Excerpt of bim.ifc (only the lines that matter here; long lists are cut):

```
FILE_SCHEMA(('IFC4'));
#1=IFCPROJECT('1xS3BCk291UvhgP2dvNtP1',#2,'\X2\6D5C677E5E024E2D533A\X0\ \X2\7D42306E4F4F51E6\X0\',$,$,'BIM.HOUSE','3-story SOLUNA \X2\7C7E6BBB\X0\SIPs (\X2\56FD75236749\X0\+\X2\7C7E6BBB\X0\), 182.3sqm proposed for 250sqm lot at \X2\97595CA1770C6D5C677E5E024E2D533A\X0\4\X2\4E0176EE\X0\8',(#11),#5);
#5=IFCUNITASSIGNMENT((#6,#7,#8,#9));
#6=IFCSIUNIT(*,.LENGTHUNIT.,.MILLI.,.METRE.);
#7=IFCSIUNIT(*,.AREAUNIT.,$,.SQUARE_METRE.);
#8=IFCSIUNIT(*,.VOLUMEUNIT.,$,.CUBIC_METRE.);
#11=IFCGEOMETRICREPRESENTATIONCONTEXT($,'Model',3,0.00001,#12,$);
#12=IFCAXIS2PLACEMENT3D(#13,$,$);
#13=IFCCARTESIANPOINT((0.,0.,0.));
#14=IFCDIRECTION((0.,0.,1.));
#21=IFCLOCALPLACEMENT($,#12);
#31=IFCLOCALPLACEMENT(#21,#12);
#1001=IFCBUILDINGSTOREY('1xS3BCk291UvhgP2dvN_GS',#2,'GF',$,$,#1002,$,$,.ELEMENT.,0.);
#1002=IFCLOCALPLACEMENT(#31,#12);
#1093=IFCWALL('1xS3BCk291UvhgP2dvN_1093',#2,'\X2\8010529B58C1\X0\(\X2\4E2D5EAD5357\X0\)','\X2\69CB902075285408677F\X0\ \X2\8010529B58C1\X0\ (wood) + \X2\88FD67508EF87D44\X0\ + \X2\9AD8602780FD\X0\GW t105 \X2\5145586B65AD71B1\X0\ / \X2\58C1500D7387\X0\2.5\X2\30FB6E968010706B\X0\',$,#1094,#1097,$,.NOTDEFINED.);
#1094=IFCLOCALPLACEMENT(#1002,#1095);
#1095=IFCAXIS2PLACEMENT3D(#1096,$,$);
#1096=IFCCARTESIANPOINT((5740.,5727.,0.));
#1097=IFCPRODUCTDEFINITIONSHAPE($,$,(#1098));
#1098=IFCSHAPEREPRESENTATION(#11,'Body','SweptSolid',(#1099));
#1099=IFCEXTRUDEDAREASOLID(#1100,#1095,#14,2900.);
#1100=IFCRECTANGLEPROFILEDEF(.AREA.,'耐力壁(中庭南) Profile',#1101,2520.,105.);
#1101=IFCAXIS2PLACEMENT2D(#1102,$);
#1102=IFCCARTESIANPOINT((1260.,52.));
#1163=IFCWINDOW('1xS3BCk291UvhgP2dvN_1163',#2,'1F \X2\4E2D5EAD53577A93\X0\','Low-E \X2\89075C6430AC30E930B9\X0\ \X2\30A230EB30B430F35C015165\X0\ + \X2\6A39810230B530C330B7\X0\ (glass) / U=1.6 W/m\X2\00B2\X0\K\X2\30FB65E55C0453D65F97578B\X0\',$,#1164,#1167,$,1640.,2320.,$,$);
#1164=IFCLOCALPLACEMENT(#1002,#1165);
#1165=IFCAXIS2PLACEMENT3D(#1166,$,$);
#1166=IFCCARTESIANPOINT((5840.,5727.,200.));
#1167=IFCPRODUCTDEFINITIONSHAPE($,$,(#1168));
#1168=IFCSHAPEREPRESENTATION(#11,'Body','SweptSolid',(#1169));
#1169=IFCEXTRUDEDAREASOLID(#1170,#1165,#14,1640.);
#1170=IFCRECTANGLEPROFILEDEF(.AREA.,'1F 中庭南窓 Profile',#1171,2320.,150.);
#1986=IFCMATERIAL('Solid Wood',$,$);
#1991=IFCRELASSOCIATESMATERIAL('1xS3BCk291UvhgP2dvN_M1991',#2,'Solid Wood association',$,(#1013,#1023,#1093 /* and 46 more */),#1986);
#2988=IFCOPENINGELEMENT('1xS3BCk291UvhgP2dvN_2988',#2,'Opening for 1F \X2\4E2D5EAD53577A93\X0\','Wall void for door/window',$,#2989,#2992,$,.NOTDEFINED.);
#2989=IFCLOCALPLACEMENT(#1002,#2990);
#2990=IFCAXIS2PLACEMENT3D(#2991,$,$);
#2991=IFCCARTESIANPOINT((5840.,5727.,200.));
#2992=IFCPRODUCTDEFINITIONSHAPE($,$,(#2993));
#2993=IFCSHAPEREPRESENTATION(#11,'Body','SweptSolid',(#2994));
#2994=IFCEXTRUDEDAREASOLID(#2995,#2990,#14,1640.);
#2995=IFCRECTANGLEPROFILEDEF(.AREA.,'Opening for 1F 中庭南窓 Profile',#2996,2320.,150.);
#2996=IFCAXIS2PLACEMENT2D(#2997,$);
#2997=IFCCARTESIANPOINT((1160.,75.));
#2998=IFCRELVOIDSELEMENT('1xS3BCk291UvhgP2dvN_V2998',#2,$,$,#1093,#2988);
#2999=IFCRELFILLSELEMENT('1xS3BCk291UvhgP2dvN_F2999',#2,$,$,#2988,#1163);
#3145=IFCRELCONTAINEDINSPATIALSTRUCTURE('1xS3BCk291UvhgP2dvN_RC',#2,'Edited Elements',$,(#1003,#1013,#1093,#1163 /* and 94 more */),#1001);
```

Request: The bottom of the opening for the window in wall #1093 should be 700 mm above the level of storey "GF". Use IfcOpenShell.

```python
import numpy as np
import ifcopenshell
import ifcopenshell.api.geometry
import ifcopenshell.geom
import ifcopenshell.util.element
import ifcopenshell.util.placement
import ifcopenshell.util.shape
import ifcopenshell.util.unit

model = ifcopenshell.open("bim.ifc")
unit_scale = ifcopenshell.util.unit.calculate_unit_scale(model)

window = model.by_id(1163)
opening = window.FillsVoids[0].RelatingOpeningElement
storey = ifcopenshell.util.element.get_container(window, ifc_class="IfcBuildingStorey")
level = ifcopenshell.util.placement.get_local_placement(storey.ObjectPlacement)[2, 3]

# The opening's origin need not be at the sill, so measure its lowest point.
shape = ifcopenshell.geom.create_shape(ifcopenshell.geom.settings(), opening)
bottom = ifcopenshell.util.shape.get_shape_bottom_elevation(shape, shape.geometry) / unit_scale
dz = level + 700.0 - bottom

shift = np.array([0.0, 0.0, dz])
# The window is not placed relative to its opening, so move both.
for product in (opening, window):
    matrix = ifcopenshell.util.placement.get_local_placement(product.ObjectPlacement)
    matrix[:3, 3] += shift
    ifcopenshell.api.geometry.edit_object_placement(model, product=product, matrix=matrix, is_si=False)

print(f"moved by {dz * unit_scale:+.3f} m")

model.write("bim-out.ifc")
```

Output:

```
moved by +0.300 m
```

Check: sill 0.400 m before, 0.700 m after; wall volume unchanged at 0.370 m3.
